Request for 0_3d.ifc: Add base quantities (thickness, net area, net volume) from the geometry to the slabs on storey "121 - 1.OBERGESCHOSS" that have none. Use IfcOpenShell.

First a look at what the model holds.

```python
import ifcopenshell
import ifcopenshell.util.element
import ifcopenshell.util.unit

model = ifcopenshell.open("0_3d.ifc")
print(model.schema)
for unit_type in ("LENGTHUNIT", "AREAUNIT", "VOLUMEUNIT"):
    print(unit_type, ifcopenshell.util.unit.calculate_unit_scale(model, unit_type))
storey = next(s for s in model.by_type("IfcBuildingStorey") if s.Name == "121 - 1.OBERGESCHOSS")
slabs = [e for e in ifcopenshell.util.element.get_decomposition(storey) if e.is_a("IfcSlab")]
for e in sorted(slabs, key=lambda e: e.id()):
    print(e.id(), e.is_a(), e.Name, list(ifcopenshell.util.element.get_psets(e, qtos_only=True)), sep=" | ")
```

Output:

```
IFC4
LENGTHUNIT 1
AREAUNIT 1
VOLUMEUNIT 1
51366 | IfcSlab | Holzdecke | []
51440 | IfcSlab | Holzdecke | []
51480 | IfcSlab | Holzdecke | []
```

```python
import ifcopenshell
import ifcopenshell.api.pset
import ifcopenshell.geom
import ifcopenshell.util.element
import ifcopenshell.util.shape
import ifcopenshell.util.unit

model = ifcopenshell.open("0_3d.ifc")
unit_scale = ifcopenshell.util.unit.calculate_unit_scale(model)
area_scale = ifcopenshell.util.unit.calculate_unit_scale(model, "AREAUNIT")
volume_scale = ifcopenshell.util.unit.calculate_unit_scale(model, "VOLUMEUNIT")
settings = ifcopenshell.geom.settings()

storey = next(s for s in model.by_type("IfcBuildingStorey") if s.Name == "121 - 1.OBERGESCHOSS")
slabs = [e for e in ifcopenshell.util.element.get_decomposition(storey) if e.is_a("IfcSlab")]

for e in sorted(slabs, key=lambda e: e.id()):
    if ifcopenshell.util.element.get_psets(e, qtos_only=True, should_inherit=False):
        continue
    # Geometry comes back in metres, in the element's own axes.
    shape = ifcopenshell.geom.create_shape(settings, e)
    values = {
        "Width": ifcopenshell.util.shape.get_z(shape.geometry) / unit_scale,
        "NetArea": ifcopenshell.util.shape.get_footprint_area(shape.geometry) / area_scale,
        "NetVolume": ifcopenshell.util.shape.get_volume(shape.geometry) / volume_scale,
    }
    qto = ifcopenshell.api.pset.add_qto(model, product=e, name="Qto_SlabBaseQuantities")
    ifcopenshell.api.pset.edit_qto(model, qto=qto, properties=values)
    print(e.id(), {k: round(v, 3) for k, v in values.items()})

model.write("0_3d_edited.ifc")
```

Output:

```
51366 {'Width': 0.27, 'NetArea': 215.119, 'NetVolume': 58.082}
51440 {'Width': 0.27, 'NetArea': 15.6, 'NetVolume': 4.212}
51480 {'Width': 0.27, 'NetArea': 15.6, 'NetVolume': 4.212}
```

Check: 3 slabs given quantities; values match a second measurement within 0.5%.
